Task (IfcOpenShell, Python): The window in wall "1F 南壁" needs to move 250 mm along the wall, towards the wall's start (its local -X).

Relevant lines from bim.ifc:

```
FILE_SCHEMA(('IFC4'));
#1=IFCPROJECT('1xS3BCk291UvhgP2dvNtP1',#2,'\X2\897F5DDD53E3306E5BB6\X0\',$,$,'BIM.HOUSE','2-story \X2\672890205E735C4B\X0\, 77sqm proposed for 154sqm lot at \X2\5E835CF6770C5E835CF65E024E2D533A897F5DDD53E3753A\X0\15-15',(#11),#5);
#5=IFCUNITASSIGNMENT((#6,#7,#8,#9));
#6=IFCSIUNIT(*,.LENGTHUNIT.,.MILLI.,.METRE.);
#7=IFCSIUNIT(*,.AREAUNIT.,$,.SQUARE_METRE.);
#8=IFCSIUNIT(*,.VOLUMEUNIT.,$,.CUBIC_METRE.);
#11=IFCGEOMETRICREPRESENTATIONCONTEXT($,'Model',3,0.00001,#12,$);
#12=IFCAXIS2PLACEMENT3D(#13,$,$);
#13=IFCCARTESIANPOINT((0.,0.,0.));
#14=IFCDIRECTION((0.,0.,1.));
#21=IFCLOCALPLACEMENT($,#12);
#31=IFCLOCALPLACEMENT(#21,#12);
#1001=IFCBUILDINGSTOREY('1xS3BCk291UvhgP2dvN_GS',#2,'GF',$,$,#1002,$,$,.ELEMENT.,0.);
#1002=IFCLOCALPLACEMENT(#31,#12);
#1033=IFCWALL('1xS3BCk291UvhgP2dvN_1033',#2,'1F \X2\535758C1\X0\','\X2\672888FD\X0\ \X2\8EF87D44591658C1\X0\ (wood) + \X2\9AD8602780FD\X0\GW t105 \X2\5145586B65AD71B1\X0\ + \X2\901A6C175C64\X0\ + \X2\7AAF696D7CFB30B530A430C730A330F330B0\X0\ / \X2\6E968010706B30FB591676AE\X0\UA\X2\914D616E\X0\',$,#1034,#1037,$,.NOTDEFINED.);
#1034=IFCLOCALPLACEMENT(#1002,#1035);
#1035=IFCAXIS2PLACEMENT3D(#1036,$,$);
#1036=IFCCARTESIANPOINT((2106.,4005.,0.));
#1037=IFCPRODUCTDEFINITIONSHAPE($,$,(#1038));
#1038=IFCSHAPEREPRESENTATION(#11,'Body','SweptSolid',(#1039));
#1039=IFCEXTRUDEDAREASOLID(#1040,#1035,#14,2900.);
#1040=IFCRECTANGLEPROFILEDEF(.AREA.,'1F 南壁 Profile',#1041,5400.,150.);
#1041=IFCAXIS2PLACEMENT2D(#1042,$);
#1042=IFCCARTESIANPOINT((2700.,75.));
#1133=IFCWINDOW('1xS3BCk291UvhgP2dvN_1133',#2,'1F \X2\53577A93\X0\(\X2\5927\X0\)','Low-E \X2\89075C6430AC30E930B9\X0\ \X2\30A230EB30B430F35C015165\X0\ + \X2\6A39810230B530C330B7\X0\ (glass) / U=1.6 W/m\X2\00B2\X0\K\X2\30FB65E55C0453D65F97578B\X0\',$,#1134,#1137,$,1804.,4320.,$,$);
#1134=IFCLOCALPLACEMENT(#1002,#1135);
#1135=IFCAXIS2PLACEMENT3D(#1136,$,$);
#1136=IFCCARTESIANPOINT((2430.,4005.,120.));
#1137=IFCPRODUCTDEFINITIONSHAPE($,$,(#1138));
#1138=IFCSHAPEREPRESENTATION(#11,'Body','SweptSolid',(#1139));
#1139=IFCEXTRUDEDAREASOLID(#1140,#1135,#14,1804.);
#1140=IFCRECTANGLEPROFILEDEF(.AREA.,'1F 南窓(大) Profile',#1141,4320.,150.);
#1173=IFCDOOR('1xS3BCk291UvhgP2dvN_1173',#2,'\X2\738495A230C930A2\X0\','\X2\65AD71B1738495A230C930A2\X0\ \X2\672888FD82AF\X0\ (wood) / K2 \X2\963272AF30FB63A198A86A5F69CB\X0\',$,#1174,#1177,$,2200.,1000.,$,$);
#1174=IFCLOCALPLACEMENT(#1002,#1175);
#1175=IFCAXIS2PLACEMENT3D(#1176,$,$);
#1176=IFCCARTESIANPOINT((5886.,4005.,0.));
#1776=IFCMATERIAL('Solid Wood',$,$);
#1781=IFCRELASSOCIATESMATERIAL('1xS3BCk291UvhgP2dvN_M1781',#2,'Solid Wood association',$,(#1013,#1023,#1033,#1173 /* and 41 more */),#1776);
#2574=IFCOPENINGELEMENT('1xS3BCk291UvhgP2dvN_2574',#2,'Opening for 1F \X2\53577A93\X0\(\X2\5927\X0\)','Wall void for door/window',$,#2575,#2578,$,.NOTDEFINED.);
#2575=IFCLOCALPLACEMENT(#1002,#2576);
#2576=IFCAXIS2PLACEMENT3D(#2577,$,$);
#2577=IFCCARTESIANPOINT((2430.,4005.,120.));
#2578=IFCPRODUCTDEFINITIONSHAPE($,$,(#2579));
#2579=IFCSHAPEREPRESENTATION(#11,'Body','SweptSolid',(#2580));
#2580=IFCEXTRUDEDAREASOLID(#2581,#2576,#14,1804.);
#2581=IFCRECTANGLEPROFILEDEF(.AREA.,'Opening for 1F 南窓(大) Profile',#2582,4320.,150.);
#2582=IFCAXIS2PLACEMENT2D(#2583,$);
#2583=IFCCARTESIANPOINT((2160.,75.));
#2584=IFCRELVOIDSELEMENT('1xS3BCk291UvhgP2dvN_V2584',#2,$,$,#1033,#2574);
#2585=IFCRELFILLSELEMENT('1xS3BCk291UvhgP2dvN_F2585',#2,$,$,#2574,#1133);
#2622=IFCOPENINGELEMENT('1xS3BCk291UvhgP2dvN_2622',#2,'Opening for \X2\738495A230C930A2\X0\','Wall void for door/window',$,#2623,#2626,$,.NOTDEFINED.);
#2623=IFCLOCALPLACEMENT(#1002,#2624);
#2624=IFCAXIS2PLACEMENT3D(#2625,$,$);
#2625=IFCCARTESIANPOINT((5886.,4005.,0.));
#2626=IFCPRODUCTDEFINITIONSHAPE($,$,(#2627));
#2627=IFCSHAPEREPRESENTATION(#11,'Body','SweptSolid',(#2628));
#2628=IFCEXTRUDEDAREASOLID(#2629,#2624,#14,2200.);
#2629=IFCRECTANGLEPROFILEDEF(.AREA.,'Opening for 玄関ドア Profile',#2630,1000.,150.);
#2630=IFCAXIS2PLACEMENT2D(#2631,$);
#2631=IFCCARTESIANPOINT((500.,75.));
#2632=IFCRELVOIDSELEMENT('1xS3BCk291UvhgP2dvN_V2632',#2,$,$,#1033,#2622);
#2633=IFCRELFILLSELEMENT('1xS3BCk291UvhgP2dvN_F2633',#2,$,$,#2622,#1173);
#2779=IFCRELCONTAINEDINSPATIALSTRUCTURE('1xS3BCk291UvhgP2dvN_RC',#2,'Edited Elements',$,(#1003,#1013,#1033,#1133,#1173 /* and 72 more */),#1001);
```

```python
import ifcopenshell
import ifcopenshell.api.geometry
import ifcopenshell.util.placement
import ifcopenshell.util.unit

model = ifcopenshell.open("bim.ifc")
unit_scale = ifcopenshell.util.unit.calculate_unit_scale(model)

window = model.by_guid("1xS3BCk291UvhgP2dvN_1133")
opening = window.FillsVoids[0].RelatingOpeningElement
wall = opening.VoidsElements[0].RelatingBuildingElement

wall_matrix = ifcopenshell.util.placement.get_local_placement(wall.ObjectPlacement)
shift = wall_matrix[:3, 0] * -0.25 / unit_scale
before = ifcopenshell.util.placement.get_local_placement(window.ObjectPlacement)[:3, 3].copy()

# The window is not placed relative to its opening, so move both.
for product in (opening, window):
    matrix = ifcopenshell.util.placement.get_local_placement(product.ObjectPlacement)
    matrix[:3, 3] += shift
    ifcopenshell.api.geometry.edit_object_placement(model, product=product, matrix=matrix, is_si=False)

after = ifcopenshell.util.placement.get_local_placement(window.ObjectPlacement)[:3, 3]
print("window moved by", (after - before).round(3) + 0.0)

model.write("bim_updated.ifc")
```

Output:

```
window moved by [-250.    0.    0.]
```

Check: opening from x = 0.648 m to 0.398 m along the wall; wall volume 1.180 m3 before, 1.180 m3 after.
